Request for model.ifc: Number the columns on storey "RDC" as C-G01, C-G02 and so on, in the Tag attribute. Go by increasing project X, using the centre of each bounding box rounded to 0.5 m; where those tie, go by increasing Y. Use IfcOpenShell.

First a look at what the model holds.

```python
import ifcopenshell
import ifcopenshell.util.element
import ifcopenshell.util.placement

model = ifcopenshell.open("model.ifc")
print(model.schema)
storey = next(s for s in model.by_type("IfcBuildingStorey") if s.Name == "RDC")
columns = [e for e in ifcopenshell.util.element.get_decomposition(storey) if e.is_a("IfcColumn")]
for e in sorted(columns, key=lambda e: e.id()):
    origin = ifcopenshell.util.placement.get_local_placement(e.ObjectPlacement)[:3, 3]
    print(e.id(), e.Tag, e.Name, origin.round(2) + 0.0, sep=" | ")
```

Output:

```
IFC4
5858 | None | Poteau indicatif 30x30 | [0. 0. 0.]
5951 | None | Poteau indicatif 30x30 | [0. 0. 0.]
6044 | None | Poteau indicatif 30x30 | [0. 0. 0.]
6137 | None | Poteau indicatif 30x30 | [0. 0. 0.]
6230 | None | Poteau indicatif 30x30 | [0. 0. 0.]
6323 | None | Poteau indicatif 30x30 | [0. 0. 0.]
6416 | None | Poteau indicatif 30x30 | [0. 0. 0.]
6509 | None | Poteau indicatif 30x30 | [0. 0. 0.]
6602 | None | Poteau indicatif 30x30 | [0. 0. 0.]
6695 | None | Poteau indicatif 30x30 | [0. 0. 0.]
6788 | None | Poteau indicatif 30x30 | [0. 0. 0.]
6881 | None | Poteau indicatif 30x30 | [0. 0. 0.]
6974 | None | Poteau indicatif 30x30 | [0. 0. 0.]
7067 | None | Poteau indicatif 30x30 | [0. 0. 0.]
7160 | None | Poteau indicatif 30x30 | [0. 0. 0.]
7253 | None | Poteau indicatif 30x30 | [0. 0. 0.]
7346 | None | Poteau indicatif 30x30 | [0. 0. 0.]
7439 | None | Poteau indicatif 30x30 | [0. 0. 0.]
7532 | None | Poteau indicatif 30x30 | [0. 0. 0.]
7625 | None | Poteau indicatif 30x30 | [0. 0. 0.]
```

```python
import ifcopenshell
import ifcopenshell.geom
import ifcopenshell.util.element
import ifcopenshell.util.shape

model = ifcopenshell.open("model.ifc")
settings = ifcopenshell.geom.settings()
settings.set("use-world-coords", True)


def centre(element):
    shape = ifcopenshell.geom.create_shape(settings, element)
    return ifcopenshell.util.shape.get_bbox_centroid(shape.geometry)


storey = next(s for s in model.by_type("IfcBuildingStorey") if s.Name == "RDC")
columns = [e for e in ifcopenshell.util.element.get_decomposition(storey) if e.is_a("IfcColumn")]

# Insertion points can sit at a corner or the storey origin, so sort by the geometry (in metres).
centres = {e: centre(e) for e in columns}
columns.sort(key=lambda e: (round(centres[e][0] / 0.5), centres[e][1]))

for i, e in enumerate(columns, start=1):
    number = f"C-G{i:02d}"
    e.Tag = number
    print(e.id(), number)

model.write("model_edited.ifc")
```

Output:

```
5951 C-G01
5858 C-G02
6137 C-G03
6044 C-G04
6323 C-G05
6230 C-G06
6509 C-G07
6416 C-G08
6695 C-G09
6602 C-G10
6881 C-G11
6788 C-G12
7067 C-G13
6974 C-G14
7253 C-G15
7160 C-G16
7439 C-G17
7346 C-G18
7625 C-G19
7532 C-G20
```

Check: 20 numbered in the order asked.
